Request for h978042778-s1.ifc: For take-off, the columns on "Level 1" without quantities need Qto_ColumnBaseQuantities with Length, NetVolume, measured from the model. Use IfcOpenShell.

First a look at what the model holds.

```python
import ifcopenshell
import ifcopenshell.util.element
import ifcopenshell.util.unit

model = ifcopenshell.open("h978042778-s1.ifc")
print(model.schema)
for unit_type in ("LENGTHUNIT", "AREAUNIT", "VOLUMEUNIT"):
    print(unit_type, ifcopenshell.util.unit.calculate_unit_scale(model, unit_type))
storey = next(s for s in model.by_type("IfcBuildingStorey") if s.Name == "Level 1")
columns = [e for e in ifcopenshell.util.element.get_decomposition(storey) if e.is_a("IfcColumn")]
for e in sorted(columns, key=lambda e: e.id()):
    print(e.id(), e.is_a(), e.Name, list(ifcopenshell.util.element.get_psets(e, qtos_only=True)), sep=" | ")
```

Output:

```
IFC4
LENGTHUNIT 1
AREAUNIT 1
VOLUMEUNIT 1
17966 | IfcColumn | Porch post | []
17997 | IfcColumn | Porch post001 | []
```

```python
import ifcopenshell
import ifcopenshell.api.pset
import ifcopenshell.geom
import ifcopenshell.util.element
import ifcopenshell.util.shape
import ifcopenshell.util.unit

model = ifcopenshell.open("h978042778-s1.ifc")
unit_scale = ifcopenshell.util.unit.calculate_unit_scale(model)
volume_scale = ifcopenshell.util.unit.calculate_unit_scale(model, "VOLUMEUNIT")
settings = ifcopenshell.geom.settings()

storey = next(s for s in model.by_type("IfcBuildingStorey") if s.Name == "Level 1")
columns = [e for e in ifcopenshell.util.element.get_decomposition(storey) if e.is_a("IfcColumn")]

for e in sorted(columns, key=lambda e: e.id()):
    if ifcopenshell.util.element.get_psets(e, qtos_only=True, should_inherit=False):
        continue
    # Geometry comes back in metres, in the element's own axes.
    shape = ifcopenshell.geom.create_shape(settings, e)
    values = {
        "Length": ifcopenshell.util.shape.get_z(shape.geometry) / unit_scale,
        "NetVolume": ifcopenshell.util.shape.get_volume(shape.geometry) / volume_scale,
    }
    qto = ifcopenshell.api.pset.add_qto(model, product=e, name="Qto_ColumnBaseQuantities")
    ifcopenshell.api.pset.edit_qto(model, qto=qto, properties=values)
    print(e.id(), {k: round(v, 3) for k, v in values.items()})

model.write("h978042778-s1_v2.ifc")
```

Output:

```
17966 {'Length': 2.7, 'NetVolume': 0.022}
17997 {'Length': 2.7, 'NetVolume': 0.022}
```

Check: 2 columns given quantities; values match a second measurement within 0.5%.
